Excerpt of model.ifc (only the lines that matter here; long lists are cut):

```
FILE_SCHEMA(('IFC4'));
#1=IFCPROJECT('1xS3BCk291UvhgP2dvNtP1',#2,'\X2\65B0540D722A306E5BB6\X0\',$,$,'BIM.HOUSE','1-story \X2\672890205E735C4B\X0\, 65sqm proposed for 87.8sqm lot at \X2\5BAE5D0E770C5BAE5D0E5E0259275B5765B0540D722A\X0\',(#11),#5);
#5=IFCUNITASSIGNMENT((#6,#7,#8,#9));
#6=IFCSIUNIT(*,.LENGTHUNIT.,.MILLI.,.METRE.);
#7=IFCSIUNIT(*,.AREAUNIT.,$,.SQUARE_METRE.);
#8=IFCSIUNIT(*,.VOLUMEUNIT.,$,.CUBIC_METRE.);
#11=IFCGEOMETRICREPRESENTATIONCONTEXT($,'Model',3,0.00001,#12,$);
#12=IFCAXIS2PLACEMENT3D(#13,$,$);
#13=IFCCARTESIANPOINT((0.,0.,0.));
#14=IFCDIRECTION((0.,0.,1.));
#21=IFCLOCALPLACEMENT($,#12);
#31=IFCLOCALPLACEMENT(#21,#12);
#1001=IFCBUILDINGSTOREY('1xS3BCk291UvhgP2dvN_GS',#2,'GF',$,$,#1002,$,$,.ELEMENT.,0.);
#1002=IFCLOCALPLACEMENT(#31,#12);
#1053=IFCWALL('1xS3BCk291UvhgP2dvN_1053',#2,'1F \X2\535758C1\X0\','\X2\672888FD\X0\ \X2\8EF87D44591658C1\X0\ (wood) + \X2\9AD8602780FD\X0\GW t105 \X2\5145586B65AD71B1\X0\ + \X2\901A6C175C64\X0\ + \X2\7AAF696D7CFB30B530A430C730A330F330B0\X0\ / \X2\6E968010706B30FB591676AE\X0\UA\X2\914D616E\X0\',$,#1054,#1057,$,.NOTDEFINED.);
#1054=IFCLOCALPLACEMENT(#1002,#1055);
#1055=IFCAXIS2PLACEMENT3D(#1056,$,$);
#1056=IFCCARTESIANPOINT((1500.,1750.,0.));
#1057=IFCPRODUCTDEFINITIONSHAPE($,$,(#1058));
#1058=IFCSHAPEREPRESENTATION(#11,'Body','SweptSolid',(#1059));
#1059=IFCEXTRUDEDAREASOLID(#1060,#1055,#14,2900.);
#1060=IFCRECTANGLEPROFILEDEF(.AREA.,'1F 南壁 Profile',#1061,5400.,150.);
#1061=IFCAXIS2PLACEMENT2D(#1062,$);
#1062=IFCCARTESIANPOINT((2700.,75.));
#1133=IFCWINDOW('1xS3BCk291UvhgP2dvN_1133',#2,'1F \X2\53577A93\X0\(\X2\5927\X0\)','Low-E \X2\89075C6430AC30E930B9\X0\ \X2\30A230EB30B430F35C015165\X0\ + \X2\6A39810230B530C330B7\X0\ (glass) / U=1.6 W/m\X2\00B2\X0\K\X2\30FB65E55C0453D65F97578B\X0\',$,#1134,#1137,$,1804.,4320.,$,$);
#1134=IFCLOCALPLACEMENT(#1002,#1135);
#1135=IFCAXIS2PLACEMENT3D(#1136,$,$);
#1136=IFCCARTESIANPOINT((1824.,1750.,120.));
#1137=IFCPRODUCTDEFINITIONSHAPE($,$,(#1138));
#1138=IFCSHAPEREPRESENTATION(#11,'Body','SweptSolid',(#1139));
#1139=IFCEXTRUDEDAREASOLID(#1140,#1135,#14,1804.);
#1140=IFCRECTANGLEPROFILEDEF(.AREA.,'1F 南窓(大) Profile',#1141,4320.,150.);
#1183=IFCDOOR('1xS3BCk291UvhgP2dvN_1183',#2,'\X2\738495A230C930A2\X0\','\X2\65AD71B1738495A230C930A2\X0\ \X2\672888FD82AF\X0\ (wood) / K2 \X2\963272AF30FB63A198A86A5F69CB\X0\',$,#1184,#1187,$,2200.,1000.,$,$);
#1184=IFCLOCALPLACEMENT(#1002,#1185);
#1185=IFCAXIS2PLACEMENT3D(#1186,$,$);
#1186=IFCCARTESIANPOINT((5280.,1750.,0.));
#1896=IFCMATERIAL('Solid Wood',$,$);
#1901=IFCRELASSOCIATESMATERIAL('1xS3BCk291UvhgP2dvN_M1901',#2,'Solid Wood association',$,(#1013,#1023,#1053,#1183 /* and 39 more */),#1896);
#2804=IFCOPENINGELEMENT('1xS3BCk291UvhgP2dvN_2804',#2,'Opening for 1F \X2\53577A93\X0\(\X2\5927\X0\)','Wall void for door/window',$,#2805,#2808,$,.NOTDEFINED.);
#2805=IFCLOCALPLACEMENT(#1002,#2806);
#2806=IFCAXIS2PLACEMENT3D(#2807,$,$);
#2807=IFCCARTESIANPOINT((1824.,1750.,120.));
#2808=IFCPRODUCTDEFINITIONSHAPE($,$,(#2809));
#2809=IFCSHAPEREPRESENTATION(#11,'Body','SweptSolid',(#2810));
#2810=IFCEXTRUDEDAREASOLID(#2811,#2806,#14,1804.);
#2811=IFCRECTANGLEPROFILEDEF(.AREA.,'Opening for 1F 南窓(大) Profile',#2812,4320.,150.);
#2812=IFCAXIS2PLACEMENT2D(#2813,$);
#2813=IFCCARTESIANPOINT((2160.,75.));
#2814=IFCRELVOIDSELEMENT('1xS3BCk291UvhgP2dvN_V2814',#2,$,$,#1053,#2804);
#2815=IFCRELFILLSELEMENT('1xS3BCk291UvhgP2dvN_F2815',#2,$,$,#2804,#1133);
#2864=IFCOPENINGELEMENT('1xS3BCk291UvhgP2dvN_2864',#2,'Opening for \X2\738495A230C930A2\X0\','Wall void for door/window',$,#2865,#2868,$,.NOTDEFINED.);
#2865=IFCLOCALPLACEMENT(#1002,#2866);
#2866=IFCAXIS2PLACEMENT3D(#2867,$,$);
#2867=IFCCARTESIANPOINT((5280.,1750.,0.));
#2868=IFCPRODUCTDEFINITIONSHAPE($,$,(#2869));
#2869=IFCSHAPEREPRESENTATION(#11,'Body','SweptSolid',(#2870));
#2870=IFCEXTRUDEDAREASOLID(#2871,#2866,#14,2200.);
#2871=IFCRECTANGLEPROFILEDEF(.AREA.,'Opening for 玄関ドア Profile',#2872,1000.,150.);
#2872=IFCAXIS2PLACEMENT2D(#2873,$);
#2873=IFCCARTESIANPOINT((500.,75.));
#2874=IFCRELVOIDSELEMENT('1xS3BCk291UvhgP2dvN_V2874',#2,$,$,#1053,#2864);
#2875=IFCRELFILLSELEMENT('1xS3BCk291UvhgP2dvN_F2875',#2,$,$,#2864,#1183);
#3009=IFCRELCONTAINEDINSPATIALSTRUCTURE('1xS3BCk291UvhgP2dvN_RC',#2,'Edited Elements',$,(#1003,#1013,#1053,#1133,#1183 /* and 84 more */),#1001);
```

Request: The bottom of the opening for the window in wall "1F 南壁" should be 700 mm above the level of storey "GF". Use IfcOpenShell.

```python
import numpy as np
import ifcopenshell
import ifcopenshell.api.geometry
import ifcopenshell.geom
import ifcopenshell.util.element
import ifcopenshell.util.placement
import ifcopenshell.util.shape
import ifcopenshell.util.unit

model = ifcopenshell.open("model.ifc")
unit_scale = ifcopenshell.util.unit.calculate_unit_scale(model)

window = model.by_id(1133)
opening = window.FillsVoids[0].RelatingOpeningElement
storey = ifcopenshell.util.element.get_container(window, ifc_class="IfcBuildingStorey")
level = ifcopenshell.util.placement.get_local_placement(storey.ObjectPlacement)[2, 3]

# The opening's origin need not be at the sill, so measure its lowest point.
shape = ifcopenshell.geom.create_shape(ifcopenshell.geom.settings(), opening)
bottom = ifcopenshell.util.shape.get_shape_bottom_elevation(shape, shape.geometry) / unit_scale
dz = level + 0.7 / unit_scale - bottom

shift = np.array([0.0, 0.0, dz])
# The window is not placed relative to its opening, so move both.
for product in (opening, window):
    matrix = ifcopenshell.util.placement.get_local_placement(product.ObjectPlacement)
    matrix[:3, 3] += shift
    ifcopenshell.api.geometry.edit_object_placement(model, product=product, matrix=matrix, is_si=False)

print(f"moved by {dz * unit_scale:+.3f} m")

model.write("model_v2.ifc")
```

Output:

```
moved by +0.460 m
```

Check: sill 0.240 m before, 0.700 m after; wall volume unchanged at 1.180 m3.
